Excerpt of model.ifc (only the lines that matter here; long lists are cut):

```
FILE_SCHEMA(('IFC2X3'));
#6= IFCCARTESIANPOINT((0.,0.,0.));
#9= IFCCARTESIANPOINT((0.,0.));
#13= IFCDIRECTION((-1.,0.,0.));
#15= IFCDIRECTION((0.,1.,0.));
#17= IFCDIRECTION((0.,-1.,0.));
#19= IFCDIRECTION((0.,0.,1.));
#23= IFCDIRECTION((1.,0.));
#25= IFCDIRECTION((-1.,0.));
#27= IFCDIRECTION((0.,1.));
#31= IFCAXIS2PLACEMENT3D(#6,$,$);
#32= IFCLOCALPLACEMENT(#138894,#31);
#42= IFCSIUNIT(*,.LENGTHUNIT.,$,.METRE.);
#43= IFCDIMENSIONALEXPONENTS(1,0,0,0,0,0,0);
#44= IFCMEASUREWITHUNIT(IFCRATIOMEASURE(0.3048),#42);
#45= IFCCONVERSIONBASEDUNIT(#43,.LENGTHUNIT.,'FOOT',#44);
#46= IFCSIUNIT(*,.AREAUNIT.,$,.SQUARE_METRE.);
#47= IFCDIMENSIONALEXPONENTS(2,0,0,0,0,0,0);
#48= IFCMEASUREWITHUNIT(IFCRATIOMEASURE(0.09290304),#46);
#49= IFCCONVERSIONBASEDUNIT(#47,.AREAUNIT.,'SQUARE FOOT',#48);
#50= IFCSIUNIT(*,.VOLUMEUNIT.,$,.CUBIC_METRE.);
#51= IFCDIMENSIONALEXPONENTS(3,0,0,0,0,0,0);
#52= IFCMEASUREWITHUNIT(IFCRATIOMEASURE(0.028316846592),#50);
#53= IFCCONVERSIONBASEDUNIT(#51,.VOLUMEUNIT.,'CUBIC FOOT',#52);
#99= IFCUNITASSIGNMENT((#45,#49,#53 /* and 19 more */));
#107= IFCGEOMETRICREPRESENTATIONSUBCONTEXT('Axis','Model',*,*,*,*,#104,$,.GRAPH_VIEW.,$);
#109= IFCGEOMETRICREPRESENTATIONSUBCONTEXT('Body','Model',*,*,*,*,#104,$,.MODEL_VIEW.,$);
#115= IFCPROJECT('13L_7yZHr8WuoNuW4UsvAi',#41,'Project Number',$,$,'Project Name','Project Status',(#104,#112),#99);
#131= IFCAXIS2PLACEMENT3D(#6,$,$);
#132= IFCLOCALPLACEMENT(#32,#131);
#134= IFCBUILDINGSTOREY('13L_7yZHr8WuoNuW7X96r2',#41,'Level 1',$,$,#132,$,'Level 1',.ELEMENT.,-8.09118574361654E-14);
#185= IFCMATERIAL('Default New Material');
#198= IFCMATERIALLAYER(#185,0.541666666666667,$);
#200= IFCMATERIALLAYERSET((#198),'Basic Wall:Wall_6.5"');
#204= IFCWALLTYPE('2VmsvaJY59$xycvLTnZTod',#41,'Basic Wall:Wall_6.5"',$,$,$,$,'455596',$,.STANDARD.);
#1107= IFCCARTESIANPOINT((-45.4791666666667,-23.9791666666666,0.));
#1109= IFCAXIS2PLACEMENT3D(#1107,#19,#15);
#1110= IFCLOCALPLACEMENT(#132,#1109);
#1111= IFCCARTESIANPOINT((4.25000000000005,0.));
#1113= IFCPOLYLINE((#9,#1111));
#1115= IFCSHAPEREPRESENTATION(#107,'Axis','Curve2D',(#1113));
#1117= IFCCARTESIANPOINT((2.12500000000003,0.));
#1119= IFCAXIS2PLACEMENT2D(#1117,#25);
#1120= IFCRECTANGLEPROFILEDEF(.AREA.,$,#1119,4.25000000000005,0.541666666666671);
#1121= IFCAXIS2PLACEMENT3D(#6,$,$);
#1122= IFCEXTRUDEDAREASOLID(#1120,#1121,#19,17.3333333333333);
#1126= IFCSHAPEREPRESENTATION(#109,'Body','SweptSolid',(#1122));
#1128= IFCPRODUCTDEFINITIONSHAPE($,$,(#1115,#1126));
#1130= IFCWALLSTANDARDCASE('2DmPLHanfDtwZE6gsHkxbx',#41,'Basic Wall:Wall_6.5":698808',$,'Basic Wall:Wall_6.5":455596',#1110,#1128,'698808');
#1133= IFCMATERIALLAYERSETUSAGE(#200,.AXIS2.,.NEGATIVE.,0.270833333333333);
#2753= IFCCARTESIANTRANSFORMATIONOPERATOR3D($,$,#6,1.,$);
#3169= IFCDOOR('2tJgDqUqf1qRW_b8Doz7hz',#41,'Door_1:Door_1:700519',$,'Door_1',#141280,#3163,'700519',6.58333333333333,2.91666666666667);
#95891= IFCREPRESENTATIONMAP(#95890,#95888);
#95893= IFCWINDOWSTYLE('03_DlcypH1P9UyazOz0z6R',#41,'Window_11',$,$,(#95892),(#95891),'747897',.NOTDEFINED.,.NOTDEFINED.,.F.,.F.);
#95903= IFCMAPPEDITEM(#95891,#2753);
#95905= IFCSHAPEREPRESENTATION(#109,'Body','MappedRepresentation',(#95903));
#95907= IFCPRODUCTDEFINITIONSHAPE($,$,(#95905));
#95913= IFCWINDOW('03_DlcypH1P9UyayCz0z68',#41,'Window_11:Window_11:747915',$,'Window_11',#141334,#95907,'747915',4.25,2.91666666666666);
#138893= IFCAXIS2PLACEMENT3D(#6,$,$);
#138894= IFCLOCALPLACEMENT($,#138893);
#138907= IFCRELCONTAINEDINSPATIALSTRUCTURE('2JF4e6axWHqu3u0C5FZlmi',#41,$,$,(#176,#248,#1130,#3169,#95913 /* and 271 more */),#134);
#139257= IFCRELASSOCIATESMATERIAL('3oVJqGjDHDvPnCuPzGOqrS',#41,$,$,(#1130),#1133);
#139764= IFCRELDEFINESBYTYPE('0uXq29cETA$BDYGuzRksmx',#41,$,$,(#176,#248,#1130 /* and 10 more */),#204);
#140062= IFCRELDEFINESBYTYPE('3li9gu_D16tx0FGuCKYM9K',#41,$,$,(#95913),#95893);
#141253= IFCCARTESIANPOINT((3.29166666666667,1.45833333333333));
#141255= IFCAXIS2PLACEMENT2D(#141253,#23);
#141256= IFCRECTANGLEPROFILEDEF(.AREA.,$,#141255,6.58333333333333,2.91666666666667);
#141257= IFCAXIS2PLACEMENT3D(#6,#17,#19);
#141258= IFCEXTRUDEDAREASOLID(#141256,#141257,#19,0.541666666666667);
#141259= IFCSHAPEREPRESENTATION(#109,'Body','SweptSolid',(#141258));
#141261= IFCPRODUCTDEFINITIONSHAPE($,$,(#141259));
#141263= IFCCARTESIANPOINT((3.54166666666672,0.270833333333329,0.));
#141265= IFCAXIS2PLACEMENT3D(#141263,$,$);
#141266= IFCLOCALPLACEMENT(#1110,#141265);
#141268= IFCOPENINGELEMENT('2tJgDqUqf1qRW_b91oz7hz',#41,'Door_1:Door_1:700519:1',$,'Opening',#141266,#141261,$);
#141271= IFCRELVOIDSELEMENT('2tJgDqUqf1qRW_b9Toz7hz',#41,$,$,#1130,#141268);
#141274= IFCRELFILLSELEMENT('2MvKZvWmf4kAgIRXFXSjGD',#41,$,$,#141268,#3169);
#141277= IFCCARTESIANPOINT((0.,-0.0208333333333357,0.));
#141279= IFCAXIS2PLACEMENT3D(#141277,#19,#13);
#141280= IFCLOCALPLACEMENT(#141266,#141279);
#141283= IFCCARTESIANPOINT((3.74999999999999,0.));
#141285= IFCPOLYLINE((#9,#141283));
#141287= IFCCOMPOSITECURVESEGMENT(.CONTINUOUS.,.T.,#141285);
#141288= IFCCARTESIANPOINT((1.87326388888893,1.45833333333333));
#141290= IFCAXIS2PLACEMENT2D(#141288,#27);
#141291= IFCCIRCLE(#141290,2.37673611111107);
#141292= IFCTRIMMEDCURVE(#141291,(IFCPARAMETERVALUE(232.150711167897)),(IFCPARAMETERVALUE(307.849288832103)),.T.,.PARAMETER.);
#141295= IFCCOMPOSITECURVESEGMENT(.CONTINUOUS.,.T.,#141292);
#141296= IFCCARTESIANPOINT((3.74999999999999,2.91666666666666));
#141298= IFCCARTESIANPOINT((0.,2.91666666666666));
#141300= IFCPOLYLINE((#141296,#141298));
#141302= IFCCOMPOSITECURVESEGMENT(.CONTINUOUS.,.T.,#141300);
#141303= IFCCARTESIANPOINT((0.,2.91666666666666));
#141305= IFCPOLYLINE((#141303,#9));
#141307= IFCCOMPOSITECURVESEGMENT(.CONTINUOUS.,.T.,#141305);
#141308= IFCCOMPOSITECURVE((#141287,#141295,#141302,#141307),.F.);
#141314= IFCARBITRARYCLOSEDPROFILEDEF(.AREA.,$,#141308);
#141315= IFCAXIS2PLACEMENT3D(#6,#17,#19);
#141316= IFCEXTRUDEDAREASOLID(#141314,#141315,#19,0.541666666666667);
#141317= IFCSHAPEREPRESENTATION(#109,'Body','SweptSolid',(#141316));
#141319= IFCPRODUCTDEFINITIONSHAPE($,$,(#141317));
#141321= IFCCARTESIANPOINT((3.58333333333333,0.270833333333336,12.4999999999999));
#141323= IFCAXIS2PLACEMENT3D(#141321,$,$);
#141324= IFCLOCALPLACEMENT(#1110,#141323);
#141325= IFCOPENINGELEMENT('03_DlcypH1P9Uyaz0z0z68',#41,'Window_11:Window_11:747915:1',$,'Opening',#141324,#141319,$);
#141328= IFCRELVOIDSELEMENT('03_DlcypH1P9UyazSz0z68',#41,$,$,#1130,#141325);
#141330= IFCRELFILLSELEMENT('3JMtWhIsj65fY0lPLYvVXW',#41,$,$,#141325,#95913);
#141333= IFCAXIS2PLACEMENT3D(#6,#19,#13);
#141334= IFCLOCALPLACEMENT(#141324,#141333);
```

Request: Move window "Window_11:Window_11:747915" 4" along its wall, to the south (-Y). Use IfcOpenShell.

```python
import ifcopenshell
import ifcopenshell.api.geometry
import ifcopenshell.util.placement
import ifcopenshell.util.unit

model = ifcopenshell.open("model.ifc")
unit_scale = ifcopenshell.util.unit.calculate_unit_scale(model)

window = model.by_id(95913)
opening = window.FillsVoids[0].RelatingOpeningElement
wall = opening.VoidsElements[0].RelatingBuildingElement

wall_matrix = ifcopenshell.util.placement.get_local_placement(wall.ObjectPlacement)
shift = wall_matrix[:3, 0] * -4 * 0.0254 / unit_scale
before = ifcopenshell.util.placement.get_local_placement(window.ObjectPlacement)[:3, 3].copy()

# The window is placed relative to its opening, so it follows when the opening moves.
matrix = ifcopenshell.util.placement.get_local_placement(opening.ObjectPlacement)
matrix[:3, 3] += shift
ifcopenshell.api.geometry.edit_object_placement(
    model, product=opening, matrix=matrix, is_si=False, should_transform_children=True
)

after = ifcopenshell.util.placement.get_local_placement(window.ObjectPlacement)[:3, 3]
print("window moved by", (after - before).round(3) + 0.0)

model.write("model_v2.ifc")
```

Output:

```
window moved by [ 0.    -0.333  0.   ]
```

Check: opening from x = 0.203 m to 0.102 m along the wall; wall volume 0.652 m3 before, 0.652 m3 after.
